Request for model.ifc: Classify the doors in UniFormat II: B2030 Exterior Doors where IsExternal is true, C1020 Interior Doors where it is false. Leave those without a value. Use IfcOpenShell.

First a look at what the model holds.

```python
import ifcopenshell
import ifcopenshell.util.element

model = ifcopenshell.open("model.ifc")
print(model.schema)
print("classifications:", [c.Name for c in model.by_type("IfcClassification")])
values = [ifcopenshell.util.element.get_pset(e, "Pset_DoorCommon", "IsExternal") for e in model.by_type("IfcDoor")]
for value in (True, False, None):
    print("IsExternal", value, values.count(value))
```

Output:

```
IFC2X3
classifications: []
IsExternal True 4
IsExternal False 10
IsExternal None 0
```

```python
import ifcopenshell
import ifcopenshell.api.classification
import ifcopenshell.util.element

model = ifcopenshell.open("model.ifc")

# IFC2X3 requires Source and Edition and has no link from the project to the system.
system = model.create_entity("IfcClassification", Source="ASTM", Edition="E1557", Name="UniFormat II")

doors = model.by_type("IfcDoor")
external = {e: ifcopenshell.util.element.get_pset(e, "Pset_DoorCommon", "IsExternal") for e in doors}
for flag, code, name in ((True, "B2030", "Exterior Doors"), (False, "C1020", "Interior Doors")):
    products = [e for e in doors if external[e] is flag]
    ifcopenshell.api.classification.add_reference(
        model, products=products, classification=system, identification=code, name=name
    )
    print(code, len(products))

model.write("model_updated.ifc")
```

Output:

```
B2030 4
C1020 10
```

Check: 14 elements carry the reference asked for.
